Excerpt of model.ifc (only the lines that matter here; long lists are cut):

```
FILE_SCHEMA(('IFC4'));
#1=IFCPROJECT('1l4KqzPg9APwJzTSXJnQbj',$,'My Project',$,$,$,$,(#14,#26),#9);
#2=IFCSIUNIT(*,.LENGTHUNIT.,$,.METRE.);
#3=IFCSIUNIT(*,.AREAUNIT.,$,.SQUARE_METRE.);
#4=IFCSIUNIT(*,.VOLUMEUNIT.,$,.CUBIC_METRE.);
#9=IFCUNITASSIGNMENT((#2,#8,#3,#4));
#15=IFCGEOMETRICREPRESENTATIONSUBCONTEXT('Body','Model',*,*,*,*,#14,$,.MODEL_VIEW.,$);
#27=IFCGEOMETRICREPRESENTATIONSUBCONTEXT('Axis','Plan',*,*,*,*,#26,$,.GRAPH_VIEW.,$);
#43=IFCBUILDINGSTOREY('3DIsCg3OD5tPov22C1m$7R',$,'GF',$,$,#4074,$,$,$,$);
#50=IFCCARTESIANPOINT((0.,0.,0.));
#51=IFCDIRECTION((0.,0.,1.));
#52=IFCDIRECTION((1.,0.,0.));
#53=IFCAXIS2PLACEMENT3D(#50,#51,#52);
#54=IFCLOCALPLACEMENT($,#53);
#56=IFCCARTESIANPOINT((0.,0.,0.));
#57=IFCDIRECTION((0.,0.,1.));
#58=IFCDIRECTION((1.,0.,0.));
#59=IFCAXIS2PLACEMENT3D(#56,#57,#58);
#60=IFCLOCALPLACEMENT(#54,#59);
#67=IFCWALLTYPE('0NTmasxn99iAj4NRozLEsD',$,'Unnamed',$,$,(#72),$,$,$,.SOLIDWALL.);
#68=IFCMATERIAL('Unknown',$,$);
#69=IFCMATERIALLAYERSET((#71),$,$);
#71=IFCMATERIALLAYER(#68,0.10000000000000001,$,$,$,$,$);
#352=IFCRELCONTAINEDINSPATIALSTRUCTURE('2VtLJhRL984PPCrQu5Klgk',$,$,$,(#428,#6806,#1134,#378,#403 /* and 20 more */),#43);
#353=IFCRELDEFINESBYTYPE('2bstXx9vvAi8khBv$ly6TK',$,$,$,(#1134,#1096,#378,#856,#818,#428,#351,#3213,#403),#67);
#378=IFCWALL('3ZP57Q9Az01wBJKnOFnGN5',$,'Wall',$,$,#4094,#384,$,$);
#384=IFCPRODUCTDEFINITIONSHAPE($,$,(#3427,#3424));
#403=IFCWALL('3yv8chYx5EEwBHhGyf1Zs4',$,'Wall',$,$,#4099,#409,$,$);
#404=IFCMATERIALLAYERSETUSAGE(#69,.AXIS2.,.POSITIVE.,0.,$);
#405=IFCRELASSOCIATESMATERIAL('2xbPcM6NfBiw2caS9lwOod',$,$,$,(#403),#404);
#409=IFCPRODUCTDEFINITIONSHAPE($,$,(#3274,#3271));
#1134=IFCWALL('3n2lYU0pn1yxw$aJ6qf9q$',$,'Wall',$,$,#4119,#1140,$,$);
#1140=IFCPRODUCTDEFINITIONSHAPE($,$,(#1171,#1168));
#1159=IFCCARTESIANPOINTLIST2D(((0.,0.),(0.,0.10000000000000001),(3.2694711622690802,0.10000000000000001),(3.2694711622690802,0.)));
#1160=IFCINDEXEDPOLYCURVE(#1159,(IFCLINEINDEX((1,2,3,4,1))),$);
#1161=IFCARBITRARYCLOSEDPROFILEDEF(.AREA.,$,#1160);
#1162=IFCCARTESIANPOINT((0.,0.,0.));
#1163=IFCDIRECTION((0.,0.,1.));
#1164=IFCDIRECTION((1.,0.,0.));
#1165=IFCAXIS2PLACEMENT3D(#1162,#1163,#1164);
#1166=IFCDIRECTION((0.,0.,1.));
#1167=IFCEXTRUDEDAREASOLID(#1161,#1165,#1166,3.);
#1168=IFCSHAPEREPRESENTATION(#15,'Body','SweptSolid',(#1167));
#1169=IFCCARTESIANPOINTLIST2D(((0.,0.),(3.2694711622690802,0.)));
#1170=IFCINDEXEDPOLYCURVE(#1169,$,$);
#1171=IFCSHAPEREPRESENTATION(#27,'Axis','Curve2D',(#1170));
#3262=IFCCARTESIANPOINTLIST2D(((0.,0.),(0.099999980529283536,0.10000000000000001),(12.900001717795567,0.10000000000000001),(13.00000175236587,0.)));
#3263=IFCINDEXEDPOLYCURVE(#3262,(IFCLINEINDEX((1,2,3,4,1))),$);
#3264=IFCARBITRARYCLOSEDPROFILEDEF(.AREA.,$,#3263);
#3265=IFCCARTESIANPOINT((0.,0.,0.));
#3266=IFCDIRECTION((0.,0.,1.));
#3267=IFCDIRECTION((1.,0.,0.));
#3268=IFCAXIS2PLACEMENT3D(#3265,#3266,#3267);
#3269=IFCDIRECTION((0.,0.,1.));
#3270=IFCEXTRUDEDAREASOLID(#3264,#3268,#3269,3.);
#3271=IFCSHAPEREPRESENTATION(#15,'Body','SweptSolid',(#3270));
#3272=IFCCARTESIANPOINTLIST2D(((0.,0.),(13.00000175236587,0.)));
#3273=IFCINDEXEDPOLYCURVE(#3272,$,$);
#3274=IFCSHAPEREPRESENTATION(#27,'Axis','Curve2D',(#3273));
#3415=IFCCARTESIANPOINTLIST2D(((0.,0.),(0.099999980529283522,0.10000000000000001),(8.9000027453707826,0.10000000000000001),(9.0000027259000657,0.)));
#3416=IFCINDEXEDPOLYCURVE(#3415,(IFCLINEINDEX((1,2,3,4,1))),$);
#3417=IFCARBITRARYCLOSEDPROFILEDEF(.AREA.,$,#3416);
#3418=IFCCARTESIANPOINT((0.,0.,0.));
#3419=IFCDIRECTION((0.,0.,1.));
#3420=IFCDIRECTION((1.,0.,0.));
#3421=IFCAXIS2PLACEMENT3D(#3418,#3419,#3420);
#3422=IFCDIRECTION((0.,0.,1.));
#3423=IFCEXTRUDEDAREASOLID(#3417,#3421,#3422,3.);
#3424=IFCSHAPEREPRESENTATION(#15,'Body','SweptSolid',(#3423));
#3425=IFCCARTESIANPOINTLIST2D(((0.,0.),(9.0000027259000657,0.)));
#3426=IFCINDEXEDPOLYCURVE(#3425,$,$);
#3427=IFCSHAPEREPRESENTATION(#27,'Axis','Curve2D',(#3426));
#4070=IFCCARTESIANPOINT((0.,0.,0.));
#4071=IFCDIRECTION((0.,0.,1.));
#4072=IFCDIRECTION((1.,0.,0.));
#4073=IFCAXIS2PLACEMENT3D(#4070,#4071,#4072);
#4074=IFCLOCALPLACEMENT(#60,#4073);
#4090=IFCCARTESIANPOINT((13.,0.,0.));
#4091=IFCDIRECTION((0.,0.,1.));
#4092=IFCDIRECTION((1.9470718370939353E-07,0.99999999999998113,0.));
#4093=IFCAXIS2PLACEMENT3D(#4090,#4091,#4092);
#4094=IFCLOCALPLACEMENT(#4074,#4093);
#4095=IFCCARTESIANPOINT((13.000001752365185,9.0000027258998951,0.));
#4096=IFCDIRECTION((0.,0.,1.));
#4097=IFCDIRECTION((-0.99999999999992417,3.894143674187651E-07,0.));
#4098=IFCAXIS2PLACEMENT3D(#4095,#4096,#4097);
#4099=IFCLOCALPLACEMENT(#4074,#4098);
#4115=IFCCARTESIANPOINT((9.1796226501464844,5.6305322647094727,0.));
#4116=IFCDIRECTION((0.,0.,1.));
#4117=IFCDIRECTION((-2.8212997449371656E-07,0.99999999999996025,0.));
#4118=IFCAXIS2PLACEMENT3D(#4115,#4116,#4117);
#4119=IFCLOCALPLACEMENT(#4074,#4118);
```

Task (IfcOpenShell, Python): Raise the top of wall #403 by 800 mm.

```python
import ifcopenshell
import ifcopenshell.geom
import ifcopenshell.util.representation
import ifcopenshell.util.shape

model = ifcopenshell.open("model.ifc")
settings = ifcopenshell.geom.settings()


def volume(element):
    """Net volume in cubic metres, openings subtracted."""
    shape = ifcopenshell.geom.create_shape(settings, element)
    return ifcopenshell.util.shape.get_volume(shape.geometry)


wall = model.by_guid("3yv8chYx5EEwBHhGyf1Zs4")
before = volume(wall)

body = ifcopenshell.util.representation.get_representation(wall, "Model", "Body")
solid = body.Items[0]
old_height = solid.Depth
solid.Depth += 0.8
after = volume(wall)

print(f"height {old_height:g} -> {solid.Depth:g}, volume {before:.3f} -> {after:.3f} m3")

model.write("model_updated.ifc")
```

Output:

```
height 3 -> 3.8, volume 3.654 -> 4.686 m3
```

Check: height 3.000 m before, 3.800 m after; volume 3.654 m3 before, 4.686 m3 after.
